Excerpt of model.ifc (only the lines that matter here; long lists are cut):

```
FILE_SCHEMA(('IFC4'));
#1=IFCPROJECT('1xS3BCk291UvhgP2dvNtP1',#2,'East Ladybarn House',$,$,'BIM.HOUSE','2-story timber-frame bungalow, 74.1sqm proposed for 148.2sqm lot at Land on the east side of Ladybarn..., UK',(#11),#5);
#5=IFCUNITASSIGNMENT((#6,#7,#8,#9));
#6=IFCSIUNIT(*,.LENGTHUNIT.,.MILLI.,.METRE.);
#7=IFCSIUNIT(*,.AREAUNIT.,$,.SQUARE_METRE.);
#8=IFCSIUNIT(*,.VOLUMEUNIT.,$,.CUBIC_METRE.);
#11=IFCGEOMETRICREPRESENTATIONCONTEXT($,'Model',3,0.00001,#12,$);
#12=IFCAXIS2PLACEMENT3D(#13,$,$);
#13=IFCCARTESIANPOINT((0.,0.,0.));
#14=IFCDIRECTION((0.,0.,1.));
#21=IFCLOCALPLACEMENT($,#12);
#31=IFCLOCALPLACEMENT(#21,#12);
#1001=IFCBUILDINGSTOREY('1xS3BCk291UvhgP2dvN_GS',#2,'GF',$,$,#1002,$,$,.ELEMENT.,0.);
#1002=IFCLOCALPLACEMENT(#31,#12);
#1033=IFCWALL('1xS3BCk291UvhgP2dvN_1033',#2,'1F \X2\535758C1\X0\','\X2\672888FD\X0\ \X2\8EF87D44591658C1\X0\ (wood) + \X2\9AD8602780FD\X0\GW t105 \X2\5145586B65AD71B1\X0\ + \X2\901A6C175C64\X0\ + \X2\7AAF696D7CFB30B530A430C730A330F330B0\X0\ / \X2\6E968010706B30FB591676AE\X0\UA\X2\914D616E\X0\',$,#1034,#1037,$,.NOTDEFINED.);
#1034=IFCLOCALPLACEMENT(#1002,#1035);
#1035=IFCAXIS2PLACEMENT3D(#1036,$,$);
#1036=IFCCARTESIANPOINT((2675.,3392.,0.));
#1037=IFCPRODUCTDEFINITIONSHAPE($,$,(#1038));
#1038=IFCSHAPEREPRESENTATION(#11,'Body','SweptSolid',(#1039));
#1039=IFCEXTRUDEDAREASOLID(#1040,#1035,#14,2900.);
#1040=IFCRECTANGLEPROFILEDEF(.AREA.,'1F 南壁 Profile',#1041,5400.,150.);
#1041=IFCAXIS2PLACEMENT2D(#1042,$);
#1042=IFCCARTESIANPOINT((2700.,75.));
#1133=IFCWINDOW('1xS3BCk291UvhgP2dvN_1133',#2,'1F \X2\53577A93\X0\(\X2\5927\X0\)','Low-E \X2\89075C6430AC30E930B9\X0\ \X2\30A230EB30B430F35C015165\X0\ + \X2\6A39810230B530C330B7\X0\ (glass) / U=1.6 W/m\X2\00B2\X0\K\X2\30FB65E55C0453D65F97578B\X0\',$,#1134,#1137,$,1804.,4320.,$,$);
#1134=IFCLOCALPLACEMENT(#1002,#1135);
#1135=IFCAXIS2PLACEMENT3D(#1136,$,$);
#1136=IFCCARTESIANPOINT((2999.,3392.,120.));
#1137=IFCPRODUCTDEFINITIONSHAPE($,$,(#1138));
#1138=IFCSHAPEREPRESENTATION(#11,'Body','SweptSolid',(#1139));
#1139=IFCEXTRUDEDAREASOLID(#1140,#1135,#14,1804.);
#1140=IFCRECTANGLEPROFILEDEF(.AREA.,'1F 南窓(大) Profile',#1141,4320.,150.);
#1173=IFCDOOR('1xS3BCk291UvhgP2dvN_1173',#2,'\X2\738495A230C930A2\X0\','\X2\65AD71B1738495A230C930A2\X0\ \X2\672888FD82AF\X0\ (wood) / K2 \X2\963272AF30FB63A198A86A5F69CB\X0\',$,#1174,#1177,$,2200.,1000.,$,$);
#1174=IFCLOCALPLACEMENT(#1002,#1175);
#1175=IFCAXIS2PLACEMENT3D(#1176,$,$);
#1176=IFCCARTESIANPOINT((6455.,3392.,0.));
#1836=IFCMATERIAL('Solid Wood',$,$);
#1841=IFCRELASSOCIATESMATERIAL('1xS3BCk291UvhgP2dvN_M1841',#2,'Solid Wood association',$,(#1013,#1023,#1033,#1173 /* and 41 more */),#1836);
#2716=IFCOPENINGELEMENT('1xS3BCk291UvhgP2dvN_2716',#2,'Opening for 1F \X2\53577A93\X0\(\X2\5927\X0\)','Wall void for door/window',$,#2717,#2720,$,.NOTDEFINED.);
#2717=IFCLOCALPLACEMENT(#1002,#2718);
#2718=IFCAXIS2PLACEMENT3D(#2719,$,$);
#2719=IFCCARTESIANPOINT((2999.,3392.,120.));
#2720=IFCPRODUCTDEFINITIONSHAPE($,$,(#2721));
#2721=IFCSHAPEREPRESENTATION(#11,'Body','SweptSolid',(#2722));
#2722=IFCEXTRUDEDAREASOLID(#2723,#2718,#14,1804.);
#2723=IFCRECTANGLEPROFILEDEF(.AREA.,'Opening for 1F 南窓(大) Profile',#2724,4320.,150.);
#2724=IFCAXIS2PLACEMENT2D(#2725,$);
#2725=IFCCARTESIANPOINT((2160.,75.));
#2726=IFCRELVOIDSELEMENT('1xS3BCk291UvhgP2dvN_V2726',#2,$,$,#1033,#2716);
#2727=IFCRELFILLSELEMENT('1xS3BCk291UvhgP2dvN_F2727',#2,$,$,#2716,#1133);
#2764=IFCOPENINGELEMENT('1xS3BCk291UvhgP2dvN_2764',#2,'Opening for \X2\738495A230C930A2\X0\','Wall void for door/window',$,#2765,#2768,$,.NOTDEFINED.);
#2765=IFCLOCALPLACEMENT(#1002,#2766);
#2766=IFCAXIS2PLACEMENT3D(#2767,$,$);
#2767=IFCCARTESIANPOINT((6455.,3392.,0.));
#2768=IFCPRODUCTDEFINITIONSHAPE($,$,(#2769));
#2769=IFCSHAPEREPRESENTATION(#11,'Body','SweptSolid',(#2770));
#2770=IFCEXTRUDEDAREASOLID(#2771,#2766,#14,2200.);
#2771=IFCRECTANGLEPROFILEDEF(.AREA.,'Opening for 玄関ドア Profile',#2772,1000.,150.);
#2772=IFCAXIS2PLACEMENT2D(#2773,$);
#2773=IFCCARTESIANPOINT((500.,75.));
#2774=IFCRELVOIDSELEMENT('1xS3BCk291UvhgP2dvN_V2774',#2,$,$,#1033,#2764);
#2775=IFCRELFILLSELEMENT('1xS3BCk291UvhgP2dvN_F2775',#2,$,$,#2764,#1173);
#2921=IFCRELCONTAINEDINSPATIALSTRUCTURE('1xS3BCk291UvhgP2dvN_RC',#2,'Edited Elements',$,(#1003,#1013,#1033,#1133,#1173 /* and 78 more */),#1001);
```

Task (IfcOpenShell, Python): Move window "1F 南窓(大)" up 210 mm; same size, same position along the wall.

```python
import numpy as np
import ifcopenshell
import ifcopenshell.api.geometry
import ifcopenshell.util.placement
import ifcopenshell.util.unit

model = ifcopenshell.open("model.ifc")
unit_scale = ifcopenshell.util.unit.calculate_unit_scale(model)

window = model.by_guid("1xS3BCk291UvhgP2dvN_1133")
opening = window.FillsVoids[0].RelatingOpeningElement
dz = 0.21 / unit_scale

shift = np.array([0.0, 0.0, dz])
# The window is not placed relative to its opening, so move both.
for product in (opening, window):
    matrix = ifcopenshell.util.placement.get_local_placement(product.ObjectPlacement)
    matrix[:3, 3] += shift
    ifcopenshell.api.geometry.edit_object_placement(model, product=product, matrix=matrix, is_si=False)

print(f"moved by {dz * unit_scale:+.3f} m")

model.write("model_edited.ifc")
```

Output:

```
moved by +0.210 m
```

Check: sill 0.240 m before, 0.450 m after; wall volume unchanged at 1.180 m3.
